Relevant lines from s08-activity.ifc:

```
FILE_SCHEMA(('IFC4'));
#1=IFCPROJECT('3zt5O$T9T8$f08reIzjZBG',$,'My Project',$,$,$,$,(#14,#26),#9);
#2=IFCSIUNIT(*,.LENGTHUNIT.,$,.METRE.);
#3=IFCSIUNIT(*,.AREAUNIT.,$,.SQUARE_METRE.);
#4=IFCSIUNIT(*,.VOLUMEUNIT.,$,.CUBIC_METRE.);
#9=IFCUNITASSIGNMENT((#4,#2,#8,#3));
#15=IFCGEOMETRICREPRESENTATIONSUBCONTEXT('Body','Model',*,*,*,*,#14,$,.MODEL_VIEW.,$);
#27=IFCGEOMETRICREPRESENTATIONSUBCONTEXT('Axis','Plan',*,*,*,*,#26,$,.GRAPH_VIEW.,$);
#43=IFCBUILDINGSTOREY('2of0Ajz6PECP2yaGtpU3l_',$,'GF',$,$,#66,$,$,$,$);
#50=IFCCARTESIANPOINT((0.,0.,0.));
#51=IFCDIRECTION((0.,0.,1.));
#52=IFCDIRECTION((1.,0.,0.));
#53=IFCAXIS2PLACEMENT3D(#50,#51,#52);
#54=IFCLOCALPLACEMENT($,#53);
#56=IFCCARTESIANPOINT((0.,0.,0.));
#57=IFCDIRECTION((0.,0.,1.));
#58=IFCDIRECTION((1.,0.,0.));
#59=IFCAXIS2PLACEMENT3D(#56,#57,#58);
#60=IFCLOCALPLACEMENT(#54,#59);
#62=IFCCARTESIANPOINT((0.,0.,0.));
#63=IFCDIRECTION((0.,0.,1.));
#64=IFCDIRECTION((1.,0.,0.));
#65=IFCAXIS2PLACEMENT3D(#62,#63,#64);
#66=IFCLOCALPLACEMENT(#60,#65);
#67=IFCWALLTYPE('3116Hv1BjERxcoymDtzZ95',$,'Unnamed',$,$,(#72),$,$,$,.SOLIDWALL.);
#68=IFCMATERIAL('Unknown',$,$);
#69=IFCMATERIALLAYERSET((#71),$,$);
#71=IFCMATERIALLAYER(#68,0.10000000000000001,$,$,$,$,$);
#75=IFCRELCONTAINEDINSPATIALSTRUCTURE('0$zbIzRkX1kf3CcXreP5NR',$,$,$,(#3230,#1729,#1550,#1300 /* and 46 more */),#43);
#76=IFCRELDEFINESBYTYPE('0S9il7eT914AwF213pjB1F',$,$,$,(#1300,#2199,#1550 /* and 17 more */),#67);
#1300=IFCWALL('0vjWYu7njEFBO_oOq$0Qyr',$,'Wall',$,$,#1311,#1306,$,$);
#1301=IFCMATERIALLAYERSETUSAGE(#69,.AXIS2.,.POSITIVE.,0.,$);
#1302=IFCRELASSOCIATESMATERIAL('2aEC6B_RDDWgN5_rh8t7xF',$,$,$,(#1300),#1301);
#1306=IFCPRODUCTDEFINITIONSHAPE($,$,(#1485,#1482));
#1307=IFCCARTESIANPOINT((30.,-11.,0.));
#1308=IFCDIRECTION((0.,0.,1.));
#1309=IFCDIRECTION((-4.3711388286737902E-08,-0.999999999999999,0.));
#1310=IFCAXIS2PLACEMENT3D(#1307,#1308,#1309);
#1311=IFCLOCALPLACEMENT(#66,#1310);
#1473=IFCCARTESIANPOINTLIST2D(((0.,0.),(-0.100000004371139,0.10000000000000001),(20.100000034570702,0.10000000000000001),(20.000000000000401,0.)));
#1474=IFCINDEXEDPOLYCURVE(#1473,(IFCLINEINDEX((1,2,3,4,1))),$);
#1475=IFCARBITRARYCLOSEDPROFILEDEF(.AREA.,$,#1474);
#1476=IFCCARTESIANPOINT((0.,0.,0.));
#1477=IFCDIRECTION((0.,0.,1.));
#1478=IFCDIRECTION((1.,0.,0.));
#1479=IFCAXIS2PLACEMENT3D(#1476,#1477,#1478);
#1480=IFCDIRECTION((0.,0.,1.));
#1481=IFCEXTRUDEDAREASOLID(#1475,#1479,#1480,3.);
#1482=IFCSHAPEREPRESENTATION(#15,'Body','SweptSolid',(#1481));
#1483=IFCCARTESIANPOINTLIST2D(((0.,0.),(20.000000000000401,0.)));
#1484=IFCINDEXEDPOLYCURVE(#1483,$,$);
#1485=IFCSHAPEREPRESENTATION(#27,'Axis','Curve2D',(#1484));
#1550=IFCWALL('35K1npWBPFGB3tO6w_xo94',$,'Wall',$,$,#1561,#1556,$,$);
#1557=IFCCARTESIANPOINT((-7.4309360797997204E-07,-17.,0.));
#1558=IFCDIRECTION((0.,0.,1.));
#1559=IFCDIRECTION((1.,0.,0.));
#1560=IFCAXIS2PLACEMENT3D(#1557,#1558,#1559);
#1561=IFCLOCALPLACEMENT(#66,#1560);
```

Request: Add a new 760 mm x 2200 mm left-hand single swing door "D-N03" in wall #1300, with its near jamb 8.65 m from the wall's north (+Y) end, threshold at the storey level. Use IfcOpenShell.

```python
import numpy as np
import ifcopenshell
import ifcopenshell.api.feature
import ifcopenshell.api.geometry
import ifcopenshell.api.root
import ifcopenshell.api.spatial
import ifcopenshell.geom
import ifcopenshell.util.element
import ifcopenshell.util.placement
import ifcopenshell.util.representation
import ifcopenshell.util.shape
import ifcopenshell.util.unit

model = ifcopenshell.open("s08-activity.ifc")
unit_scale = ifcopenshell.util.unit.calculate_unit_scale(model)
settings = ifcopenshell.geom.settings()


def volume(element):
    """Net volume in cubic metres, openings subtracted."""
    shape = ifcopenshell.geom.create_shape(settings, element)
    return ifcopenshell.util.shape.get_volume(shape.geometry)


wall = model.by_guid("0vjWYu7njEFBO_oOq$0Qyr")
storey = ifcopenshell.util.element.get_container(wall, ifc_class="IfcBuildingStorey")
context = ifcopenshell.util.representation.get_context(model, "Model", "Body", "MODEL_VIEW")
before = volume(wall)

width, height, from_end, sill = 0.76, 2.2, 8.65, 0.0  # metres

# The wall runs along its own X axis, and the end named is its -X end.
wall_shape = ifcopenshell.geom.create_shape(settings, wall)
x, y, z = ifcopenshell.util.shape.get_vertices(wall_shape.geometry).T
start = x.min() + from_end
face, thickness = float(y.min()), float(y.max() - y.min())
wall_matrix = ifcopenshell.util.placement.get_local_placement(wall.ObjectPlacement)
level = ifcopenshell.util.placement.get_local_placement(storey.ObjectPlacement)[2, 3]


def in_wall(x, y):
    """Placement at x, y metres in the wall's axes, at sill height."""
    matrix = wall_matrix.copy()
    matrix[:, 3] = wall_matrix @ np.array([x / unit_scale, y / unit_scale, 0.0, 1.0])
    matrix[2, 3] = level + sill / unit_scale
    return matrix


# Opening: a box that overshoots both wall faces by 50 mm.
opening = ifcopenshell.api.root.create_entity(model, ifc_class="IfcOpeningElement", predefined_type="OPENING")
box = ifcopenshell.api.geometry.add_wall_representation(
    model, context=context, length=width, height=height, thickness=thickness + 0.1
)
ifcopenshell.api.geometry.assign_representation(model, product=opening, representation=box)
ifcopenshell.api.geometry.edit_object_placement(model, product=opening, matrix=in_wall(start, face - 0.05), is_si=False)
ifcopenshell.api.feature.add_feature(model, feature=opening, element=wall)

door = ifcopenshell.api.root.create_entity(model, ifc_class="IfcDoor", name="D-N03", predefined_type="DOOR")
door.OverallWidth, door.OverallHeight = width / unit_scale, height / unit_scale
door.OperationType = "SINGLE_SWING_LEFT"
body = ifcopenshell.api.geometry.add_door_representation(
    model,
    context=context,
    overall_width=door.OverallWidth,
    overall_height=door.OverallHeight,
    operation_type="SINGLE_SWING_LEFT",
    lining_properties={"LiningDepth": thickness / unit_scale, "ThresholdDepth": thickness / unit_scale},
)
ifcopenshell.api.geometry.assign_representation(model, product=door, representation=body)
ifcopenshell.api.spatial.assign_container(model, products=[door], relating_structure=storey)
ifcopenshell.api.feature.add_filling(model, opening=opening, element=door)

# The lining spans the wall, so the door starts at the wall face.
ifcopenshell.api.geometry.edit_object_placement(model, product=door, matrix=in_wall(start, face), is_si=False)

after = volume(wall)

print(f"wall volume {before:.3f} -> {after:.3f} m3")

model.write("s08-activity_rev.ifc")
```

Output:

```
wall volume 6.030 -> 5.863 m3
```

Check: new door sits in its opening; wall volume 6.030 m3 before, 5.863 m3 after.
